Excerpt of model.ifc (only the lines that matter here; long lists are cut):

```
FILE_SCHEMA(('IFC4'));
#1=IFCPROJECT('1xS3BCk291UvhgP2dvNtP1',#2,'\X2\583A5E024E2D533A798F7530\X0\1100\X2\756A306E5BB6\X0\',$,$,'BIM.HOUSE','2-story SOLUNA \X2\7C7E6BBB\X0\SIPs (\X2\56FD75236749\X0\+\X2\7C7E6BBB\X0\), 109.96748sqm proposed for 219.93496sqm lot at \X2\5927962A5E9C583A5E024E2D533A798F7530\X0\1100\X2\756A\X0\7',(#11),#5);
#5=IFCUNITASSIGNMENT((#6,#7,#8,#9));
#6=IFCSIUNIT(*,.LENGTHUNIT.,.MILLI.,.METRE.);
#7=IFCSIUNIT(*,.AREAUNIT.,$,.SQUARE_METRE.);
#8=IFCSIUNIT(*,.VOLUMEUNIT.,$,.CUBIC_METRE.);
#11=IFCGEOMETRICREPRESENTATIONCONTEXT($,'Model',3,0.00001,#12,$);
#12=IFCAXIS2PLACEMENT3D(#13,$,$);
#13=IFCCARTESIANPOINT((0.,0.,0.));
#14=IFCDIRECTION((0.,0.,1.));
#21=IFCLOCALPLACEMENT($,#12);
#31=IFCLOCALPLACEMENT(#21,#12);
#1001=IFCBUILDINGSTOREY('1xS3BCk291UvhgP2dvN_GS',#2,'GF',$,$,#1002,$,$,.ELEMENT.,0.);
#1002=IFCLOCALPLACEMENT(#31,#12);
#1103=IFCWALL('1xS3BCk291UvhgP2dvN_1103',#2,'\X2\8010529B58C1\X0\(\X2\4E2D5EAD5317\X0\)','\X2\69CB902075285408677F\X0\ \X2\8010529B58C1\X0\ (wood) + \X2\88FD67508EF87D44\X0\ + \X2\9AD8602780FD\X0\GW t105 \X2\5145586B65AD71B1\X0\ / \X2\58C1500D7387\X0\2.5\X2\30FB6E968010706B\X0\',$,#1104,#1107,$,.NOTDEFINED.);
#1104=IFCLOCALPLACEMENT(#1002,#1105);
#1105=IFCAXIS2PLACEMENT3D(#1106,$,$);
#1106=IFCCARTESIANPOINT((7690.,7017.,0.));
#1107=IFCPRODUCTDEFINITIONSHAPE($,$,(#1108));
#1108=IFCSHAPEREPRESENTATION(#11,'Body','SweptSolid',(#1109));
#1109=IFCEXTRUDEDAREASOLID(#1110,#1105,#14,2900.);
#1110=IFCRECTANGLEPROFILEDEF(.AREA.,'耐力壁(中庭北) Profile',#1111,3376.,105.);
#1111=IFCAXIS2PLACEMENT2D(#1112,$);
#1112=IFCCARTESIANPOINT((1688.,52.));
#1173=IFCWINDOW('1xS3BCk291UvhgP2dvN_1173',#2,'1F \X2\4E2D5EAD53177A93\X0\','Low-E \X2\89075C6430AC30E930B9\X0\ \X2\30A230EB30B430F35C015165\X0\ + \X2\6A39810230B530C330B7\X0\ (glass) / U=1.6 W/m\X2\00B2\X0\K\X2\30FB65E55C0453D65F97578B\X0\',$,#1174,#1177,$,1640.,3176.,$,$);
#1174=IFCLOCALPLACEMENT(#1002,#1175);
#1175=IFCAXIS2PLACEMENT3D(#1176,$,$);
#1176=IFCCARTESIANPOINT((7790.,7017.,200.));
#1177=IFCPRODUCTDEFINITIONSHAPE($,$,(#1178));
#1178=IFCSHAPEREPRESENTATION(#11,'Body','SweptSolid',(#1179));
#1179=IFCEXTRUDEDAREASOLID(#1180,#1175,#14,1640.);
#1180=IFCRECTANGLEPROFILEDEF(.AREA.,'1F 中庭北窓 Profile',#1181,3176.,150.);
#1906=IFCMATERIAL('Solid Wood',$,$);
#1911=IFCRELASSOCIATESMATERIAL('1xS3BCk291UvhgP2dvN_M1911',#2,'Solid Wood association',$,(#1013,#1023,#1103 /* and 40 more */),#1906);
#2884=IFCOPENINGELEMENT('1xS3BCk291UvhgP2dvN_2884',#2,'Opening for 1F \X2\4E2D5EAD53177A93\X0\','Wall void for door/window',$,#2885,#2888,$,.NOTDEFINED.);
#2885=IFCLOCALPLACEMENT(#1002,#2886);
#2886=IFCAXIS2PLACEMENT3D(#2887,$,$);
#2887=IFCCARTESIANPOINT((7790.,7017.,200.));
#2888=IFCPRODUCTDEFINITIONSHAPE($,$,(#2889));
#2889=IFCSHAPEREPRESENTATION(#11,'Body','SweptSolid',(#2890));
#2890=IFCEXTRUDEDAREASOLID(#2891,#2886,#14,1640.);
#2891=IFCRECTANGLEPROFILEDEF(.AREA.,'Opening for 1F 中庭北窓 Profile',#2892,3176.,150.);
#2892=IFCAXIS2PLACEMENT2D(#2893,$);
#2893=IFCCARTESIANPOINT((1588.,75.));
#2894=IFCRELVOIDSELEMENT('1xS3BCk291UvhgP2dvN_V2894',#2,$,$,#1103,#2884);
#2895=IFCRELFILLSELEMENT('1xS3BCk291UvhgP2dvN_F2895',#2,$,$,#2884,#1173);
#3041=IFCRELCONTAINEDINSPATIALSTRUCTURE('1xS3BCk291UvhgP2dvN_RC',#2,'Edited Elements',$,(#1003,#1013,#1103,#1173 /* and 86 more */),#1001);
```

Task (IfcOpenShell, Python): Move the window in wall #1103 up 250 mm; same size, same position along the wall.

```python
import numpy as np
import ifcopenshell
import ifcopenshell.api.geometry
import ifcopenshell.util.placement
import ifcopenshell.util.unit

model = ifcopenshell.open("model.ifc")
unit_scale = ifcopenshell.util.unit.calculate_unit_scale(model)

window = model.by_id(1173)
opening = window.FillsVoids[0].RelatingOpeningElement
dz = 250.0

shift = np.array([0.0, 0.0, dz])
# The window is not placed relative to its opening, so move both.
for product in (opening, window):
    matrix = ifcopenshell.util.placement.get_local_placement(product.ObjectPlacement)
    matrix[:3, 3] += shift
    ifcopenshell.api.geometry.edit_object_placement(model, product=product, matrix=matrix, is_si=False)

print(f"moved by {dz * unit_scale:+.3f} m")

model.write("model-out.ifc")
```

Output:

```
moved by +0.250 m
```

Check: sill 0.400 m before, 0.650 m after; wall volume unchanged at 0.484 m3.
